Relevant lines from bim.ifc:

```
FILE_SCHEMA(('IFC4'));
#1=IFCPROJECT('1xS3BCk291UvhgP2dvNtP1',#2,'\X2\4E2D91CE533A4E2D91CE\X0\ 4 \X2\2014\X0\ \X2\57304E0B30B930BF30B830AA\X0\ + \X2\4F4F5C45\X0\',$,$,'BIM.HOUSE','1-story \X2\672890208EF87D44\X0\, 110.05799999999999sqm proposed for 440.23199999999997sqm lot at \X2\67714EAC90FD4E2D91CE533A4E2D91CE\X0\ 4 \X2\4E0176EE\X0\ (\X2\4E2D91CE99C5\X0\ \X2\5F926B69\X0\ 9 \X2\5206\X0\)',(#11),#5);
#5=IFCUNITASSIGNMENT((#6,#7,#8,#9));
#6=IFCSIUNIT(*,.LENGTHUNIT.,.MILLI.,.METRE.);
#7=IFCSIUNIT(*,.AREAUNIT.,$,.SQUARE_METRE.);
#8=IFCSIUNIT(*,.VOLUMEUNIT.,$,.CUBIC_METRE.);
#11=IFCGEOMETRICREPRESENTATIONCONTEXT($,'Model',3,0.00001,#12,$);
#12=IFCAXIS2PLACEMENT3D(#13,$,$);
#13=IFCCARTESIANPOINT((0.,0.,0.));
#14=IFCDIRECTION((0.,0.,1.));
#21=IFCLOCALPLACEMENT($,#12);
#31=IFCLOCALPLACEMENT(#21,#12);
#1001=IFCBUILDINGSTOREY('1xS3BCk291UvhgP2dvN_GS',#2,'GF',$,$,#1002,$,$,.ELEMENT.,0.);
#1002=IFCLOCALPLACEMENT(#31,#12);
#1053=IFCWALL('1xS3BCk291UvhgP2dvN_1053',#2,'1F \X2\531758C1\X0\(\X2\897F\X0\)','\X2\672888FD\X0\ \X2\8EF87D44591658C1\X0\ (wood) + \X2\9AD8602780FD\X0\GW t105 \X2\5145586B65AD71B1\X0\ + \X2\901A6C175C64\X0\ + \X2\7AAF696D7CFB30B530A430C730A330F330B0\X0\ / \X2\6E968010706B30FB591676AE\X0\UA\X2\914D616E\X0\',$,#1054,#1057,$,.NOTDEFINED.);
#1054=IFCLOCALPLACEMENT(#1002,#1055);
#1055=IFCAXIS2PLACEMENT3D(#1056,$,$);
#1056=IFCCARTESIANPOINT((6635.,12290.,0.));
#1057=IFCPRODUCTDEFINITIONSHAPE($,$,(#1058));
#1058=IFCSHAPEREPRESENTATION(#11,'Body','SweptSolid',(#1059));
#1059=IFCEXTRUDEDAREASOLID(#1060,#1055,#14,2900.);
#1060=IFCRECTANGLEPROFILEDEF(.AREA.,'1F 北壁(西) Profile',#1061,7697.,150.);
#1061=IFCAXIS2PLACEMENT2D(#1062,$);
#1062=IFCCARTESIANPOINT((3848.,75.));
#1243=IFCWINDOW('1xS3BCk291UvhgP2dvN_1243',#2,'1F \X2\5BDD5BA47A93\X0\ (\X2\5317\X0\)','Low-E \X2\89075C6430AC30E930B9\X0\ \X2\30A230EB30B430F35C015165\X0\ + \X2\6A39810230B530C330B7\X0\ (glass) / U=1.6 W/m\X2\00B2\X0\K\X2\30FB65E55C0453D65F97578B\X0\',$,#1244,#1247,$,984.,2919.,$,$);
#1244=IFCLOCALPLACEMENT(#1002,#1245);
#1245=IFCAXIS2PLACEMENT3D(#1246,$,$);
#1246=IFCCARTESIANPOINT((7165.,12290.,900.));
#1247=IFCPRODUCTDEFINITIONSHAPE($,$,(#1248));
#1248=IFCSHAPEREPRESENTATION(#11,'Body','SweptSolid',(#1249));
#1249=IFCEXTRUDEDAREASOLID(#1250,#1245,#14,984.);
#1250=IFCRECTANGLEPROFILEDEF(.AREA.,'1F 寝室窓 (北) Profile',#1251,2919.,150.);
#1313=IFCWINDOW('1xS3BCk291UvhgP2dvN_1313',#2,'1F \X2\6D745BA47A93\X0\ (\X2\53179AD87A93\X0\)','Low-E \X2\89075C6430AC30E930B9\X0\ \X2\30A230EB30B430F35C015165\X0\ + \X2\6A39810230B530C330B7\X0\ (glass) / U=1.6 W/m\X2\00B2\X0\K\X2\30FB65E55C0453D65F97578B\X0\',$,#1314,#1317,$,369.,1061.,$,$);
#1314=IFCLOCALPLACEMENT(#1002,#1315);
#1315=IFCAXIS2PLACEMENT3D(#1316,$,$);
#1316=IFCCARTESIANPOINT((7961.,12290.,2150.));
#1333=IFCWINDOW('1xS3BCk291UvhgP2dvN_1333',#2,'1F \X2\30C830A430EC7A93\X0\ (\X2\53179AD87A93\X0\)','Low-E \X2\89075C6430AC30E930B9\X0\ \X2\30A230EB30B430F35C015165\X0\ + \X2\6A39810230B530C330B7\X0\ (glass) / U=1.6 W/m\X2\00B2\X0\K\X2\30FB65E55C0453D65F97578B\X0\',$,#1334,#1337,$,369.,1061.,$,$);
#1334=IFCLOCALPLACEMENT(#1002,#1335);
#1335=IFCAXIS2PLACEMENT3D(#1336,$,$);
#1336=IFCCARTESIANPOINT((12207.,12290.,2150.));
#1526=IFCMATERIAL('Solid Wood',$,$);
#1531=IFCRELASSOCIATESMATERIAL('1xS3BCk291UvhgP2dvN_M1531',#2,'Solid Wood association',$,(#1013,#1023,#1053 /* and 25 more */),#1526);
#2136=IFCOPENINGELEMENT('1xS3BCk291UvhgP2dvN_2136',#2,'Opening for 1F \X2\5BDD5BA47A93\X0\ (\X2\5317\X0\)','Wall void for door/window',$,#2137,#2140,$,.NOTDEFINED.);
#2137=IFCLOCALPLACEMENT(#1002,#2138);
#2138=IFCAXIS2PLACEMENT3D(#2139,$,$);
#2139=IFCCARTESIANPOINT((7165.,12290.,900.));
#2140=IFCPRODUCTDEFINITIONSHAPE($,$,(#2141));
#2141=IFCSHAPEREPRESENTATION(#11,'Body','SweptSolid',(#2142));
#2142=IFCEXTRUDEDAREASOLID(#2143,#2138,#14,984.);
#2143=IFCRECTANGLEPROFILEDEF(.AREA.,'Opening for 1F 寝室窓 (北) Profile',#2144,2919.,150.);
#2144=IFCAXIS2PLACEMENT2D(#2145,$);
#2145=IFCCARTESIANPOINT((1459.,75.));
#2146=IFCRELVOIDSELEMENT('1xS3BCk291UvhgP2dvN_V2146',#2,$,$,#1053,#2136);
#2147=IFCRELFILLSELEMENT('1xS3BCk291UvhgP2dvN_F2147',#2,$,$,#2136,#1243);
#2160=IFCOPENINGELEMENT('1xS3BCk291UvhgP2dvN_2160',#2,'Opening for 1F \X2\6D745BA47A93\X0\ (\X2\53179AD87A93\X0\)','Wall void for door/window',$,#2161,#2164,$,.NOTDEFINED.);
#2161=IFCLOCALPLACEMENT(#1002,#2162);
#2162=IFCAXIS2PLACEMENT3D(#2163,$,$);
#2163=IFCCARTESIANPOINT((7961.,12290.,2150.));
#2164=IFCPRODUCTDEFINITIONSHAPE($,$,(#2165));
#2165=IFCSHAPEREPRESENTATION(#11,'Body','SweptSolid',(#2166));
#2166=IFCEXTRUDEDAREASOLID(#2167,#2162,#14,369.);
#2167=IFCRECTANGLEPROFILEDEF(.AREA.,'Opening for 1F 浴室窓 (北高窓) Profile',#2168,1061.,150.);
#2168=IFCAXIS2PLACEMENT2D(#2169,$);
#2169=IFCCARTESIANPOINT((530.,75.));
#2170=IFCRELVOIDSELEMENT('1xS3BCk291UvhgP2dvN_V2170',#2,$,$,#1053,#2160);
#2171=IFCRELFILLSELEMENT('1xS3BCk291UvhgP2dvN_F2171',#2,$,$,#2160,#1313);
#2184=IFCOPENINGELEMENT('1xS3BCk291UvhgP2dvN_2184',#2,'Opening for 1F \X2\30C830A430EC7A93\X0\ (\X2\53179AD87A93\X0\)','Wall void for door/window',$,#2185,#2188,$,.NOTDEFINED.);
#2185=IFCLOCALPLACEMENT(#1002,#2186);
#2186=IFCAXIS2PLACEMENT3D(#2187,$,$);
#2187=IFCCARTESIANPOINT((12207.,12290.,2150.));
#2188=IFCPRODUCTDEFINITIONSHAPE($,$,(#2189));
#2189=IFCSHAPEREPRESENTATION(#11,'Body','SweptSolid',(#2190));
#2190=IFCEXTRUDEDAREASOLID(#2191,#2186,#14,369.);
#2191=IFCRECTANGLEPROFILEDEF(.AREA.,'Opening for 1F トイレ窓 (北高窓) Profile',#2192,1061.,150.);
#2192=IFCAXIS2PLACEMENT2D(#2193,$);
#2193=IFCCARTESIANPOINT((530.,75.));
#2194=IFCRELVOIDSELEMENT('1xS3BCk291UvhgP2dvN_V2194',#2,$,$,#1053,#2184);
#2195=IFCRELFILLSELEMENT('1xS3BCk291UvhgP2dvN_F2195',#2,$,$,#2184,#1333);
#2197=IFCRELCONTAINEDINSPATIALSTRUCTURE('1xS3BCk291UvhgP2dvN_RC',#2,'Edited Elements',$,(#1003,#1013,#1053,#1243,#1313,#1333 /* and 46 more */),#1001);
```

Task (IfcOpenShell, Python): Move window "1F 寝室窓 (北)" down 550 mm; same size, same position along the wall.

```python
import numpy as np
import ifcopenshell
import ifcopenshell.api.geometry
import ifcopenshell.util.placement
import ifcopenshell.util.unit

model = ifcopenshell.open("bim.ifc")
unit_scale = ifcopenshell.util.unit.calculate_unit_scale(model)

window = model.by_guid("1xS3BCk291UvhgP2dvN_1243")
opening = window.FillsVoids[0].RelatingOpeningElement
dz = -550.0

shift = np.array([0.0, 0.0, dz])
# The window is not placed relative to its opening, so move both.
for product in (opening, window):
    matrix = ifcopenshell.util.placement.get_local_placement(product.ObjectPlacement)
    matrix[:3, 3] += shift
    ifcopenshell.api.geometry.edit_object_placement(model, product=product, matrix=matrix, is_si=False)

print(f"moved by {dz * unit_scale:+.3f} m")

model.write("bim_rev.ifc")
```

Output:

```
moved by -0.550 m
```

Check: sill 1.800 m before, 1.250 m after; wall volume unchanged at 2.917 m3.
